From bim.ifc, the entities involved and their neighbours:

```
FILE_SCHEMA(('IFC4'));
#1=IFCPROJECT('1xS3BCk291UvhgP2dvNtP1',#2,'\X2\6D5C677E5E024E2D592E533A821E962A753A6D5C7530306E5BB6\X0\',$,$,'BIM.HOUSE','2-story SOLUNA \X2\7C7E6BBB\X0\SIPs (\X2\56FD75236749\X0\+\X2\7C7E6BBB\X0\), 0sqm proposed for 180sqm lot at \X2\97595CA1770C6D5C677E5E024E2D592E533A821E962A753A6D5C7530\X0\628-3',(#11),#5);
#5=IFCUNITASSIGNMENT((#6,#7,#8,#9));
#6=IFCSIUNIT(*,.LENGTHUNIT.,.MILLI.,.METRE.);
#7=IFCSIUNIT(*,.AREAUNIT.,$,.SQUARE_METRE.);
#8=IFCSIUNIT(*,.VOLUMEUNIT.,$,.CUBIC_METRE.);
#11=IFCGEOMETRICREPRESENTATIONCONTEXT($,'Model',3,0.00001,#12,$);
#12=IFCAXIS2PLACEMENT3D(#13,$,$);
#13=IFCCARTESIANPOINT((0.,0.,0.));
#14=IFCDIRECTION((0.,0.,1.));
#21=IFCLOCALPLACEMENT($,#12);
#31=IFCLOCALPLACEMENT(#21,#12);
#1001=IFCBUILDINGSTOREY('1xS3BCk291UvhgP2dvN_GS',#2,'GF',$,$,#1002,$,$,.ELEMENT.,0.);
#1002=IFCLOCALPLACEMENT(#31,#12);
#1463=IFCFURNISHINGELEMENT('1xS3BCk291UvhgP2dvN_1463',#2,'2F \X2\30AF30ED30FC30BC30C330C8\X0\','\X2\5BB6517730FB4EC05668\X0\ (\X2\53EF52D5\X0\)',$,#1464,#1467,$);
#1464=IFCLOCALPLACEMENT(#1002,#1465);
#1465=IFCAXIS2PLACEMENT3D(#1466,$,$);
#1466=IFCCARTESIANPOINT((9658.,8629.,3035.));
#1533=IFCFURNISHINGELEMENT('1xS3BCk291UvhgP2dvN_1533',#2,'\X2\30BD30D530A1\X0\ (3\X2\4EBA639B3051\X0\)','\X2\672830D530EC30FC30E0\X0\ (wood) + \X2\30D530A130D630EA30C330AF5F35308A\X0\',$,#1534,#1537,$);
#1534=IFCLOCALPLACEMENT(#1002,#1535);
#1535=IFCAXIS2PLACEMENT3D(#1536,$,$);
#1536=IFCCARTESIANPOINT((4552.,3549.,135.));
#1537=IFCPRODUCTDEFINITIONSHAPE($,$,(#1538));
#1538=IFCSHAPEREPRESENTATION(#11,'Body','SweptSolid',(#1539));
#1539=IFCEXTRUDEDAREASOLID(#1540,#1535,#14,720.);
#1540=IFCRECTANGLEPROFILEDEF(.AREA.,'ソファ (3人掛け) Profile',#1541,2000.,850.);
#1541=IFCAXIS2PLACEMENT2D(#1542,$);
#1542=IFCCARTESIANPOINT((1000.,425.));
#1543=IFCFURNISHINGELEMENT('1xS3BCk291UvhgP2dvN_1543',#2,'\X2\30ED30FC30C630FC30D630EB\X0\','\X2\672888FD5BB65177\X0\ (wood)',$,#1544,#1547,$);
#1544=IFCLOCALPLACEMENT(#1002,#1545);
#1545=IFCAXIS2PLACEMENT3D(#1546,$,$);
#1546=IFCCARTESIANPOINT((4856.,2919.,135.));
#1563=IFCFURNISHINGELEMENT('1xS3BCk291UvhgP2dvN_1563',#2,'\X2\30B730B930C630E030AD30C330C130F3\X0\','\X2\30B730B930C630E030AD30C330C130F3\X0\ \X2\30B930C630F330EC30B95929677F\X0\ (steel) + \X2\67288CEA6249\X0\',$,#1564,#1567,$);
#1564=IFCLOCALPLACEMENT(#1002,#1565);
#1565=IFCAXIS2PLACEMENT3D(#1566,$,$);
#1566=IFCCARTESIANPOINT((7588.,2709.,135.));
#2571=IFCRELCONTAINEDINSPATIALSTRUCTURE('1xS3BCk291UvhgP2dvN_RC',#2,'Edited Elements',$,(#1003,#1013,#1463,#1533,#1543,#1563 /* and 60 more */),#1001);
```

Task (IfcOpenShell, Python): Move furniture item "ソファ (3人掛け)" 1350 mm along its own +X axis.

```python
import ifcopenshell
import ifcopenshell.api.geometry
import ifcopenshell.util.placement
import ifcopenshell.util.unit

model = ifcopenshell.open("bim.ifc")
unit_scale = ifcopenshell.util.unit.calculate_unit_scale(model)

item = model.by_guid("1xS3BCk291UvhgP2dvN_1533")
matrix = ifcopenshell.util.placement.get_local_placement(item.ObjectPlacement)
matrix[:3, 3] += matrix[:3, 0] * 1.35 / unit_scale
ifcopenshell.api.geometry.edit_object_placement(model, product=item, matrix=matrix, is_si=False)

print(ifcopenshell.util.placement.get_local_placement(item.ObjectPlacement).round(3) + 0.0)

model.write("bim_v2.ifc")
```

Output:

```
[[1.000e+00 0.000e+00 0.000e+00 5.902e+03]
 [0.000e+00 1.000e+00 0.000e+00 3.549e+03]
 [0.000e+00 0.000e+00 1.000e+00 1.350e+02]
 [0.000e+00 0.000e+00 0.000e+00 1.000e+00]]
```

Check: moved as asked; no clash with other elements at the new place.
